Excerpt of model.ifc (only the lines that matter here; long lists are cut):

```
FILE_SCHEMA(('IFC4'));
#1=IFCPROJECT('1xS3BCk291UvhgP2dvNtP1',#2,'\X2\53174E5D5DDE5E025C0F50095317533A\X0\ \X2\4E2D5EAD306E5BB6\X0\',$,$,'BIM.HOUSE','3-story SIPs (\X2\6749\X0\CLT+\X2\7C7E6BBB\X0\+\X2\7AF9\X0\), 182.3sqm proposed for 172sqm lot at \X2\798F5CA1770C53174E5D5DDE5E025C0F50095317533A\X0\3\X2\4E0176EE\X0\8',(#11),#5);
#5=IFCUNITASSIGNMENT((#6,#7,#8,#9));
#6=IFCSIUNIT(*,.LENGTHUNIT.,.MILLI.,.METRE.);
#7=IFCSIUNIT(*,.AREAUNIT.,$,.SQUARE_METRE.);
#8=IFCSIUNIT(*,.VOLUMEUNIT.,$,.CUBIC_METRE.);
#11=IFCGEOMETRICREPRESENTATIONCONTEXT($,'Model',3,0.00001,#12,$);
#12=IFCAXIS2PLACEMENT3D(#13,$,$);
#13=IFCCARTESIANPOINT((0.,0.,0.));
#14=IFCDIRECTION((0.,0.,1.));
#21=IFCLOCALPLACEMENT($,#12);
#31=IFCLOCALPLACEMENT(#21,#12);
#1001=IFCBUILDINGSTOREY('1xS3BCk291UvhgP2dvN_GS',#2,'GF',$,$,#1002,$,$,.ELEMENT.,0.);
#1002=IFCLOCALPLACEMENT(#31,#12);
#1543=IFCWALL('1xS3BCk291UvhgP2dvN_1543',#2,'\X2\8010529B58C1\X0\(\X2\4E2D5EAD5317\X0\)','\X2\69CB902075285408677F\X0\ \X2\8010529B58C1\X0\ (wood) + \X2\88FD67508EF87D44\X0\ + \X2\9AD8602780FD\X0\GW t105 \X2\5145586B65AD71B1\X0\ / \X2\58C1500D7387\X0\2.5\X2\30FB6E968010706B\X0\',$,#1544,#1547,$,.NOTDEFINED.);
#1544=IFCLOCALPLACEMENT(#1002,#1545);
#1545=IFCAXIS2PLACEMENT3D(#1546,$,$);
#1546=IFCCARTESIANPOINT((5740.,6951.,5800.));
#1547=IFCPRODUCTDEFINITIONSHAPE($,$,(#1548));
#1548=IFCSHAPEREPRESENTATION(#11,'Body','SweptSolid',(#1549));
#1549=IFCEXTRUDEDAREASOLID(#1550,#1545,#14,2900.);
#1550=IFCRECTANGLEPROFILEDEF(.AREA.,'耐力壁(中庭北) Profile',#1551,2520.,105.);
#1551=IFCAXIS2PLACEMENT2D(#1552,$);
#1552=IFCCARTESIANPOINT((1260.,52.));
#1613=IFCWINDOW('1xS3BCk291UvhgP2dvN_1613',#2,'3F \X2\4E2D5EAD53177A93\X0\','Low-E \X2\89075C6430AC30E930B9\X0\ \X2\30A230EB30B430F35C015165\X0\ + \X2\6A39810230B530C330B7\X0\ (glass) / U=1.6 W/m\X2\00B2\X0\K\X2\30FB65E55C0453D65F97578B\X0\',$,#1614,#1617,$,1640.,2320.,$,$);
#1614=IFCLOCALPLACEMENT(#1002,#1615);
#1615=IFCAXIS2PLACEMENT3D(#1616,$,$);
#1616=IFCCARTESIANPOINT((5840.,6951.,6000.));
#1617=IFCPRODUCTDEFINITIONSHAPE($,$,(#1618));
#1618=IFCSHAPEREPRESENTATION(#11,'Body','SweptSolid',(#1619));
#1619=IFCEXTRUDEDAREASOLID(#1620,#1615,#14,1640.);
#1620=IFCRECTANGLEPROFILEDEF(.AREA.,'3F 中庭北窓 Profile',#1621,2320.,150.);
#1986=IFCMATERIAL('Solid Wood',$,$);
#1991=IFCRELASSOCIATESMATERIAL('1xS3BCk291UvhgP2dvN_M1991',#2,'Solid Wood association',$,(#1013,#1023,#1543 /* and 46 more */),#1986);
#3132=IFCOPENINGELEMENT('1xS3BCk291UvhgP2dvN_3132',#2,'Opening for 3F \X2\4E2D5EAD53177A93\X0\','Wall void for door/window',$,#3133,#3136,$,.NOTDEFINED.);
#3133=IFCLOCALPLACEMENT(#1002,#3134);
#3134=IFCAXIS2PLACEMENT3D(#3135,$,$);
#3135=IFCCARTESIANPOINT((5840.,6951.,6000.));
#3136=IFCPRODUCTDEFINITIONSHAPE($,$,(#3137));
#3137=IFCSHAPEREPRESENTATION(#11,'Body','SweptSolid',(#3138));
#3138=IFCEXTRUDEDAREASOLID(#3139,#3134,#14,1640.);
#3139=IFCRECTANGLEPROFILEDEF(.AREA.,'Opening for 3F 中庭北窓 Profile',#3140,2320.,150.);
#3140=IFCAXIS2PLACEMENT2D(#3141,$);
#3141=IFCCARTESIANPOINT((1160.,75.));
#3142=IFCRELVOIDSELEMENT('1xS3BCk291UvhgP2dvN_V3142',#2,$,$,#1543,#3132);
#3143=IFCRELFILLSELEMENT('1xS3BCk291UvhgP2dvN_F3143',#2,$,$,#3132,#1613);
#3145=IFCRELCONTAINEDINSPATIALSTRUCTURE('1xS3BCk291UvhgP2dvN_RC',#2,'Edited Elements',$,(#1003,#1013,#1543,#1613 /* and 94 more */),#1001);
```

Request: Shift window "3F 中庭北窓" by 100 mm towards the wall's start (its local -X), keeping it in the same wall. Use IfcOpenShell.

```python
import ifcopenshell
import ifcopenshell.api.geometry
import ifcopenshell.util.placement
import ifcopenshell.util.unit

model = ifcopenshell.open("model.ifc")
unit_scale = ifcopenshell.util.unit.calculate_unit_scale(model)

window = model.by_id(1613)
opening = window.FillsVoids[0].RelatingOpeningElement
wall = opening.VoidsElements[0].RelatingBuildingElement

wall_matrix = ifcopenshell.util.placement.get_local_placement(wall.ObjectPlacement)
shift = wall_matrix[:3, 0] * -0.1 / unit_scale
before = ifcopenshell.util.placement.get_local_placement(window.ObjectPlacement)[:3, 3].copy()

# The window is not placed relative to its opening, so move both.
for product in (opening, window):
    matrix = ifcopenshell.util.placement.get_local_placement(product.ObjectPlacement)
    matrix[:3, 3] += shift
    ifcopenshell.api.geometry.edit_object_placement(model, product=product, matrix=matrix, is_si=False)

after = ifcopenshell.util.placement.get_local_placement(window.ObjectPlacement)[:3, 3]
print("window moved by", (after - before).round(3) + 0.0)

model.write("model_v2.ifc")
```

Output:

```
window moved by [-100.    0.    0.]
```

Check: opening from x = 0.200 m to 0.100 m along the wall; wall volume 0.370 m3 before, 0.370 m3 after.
